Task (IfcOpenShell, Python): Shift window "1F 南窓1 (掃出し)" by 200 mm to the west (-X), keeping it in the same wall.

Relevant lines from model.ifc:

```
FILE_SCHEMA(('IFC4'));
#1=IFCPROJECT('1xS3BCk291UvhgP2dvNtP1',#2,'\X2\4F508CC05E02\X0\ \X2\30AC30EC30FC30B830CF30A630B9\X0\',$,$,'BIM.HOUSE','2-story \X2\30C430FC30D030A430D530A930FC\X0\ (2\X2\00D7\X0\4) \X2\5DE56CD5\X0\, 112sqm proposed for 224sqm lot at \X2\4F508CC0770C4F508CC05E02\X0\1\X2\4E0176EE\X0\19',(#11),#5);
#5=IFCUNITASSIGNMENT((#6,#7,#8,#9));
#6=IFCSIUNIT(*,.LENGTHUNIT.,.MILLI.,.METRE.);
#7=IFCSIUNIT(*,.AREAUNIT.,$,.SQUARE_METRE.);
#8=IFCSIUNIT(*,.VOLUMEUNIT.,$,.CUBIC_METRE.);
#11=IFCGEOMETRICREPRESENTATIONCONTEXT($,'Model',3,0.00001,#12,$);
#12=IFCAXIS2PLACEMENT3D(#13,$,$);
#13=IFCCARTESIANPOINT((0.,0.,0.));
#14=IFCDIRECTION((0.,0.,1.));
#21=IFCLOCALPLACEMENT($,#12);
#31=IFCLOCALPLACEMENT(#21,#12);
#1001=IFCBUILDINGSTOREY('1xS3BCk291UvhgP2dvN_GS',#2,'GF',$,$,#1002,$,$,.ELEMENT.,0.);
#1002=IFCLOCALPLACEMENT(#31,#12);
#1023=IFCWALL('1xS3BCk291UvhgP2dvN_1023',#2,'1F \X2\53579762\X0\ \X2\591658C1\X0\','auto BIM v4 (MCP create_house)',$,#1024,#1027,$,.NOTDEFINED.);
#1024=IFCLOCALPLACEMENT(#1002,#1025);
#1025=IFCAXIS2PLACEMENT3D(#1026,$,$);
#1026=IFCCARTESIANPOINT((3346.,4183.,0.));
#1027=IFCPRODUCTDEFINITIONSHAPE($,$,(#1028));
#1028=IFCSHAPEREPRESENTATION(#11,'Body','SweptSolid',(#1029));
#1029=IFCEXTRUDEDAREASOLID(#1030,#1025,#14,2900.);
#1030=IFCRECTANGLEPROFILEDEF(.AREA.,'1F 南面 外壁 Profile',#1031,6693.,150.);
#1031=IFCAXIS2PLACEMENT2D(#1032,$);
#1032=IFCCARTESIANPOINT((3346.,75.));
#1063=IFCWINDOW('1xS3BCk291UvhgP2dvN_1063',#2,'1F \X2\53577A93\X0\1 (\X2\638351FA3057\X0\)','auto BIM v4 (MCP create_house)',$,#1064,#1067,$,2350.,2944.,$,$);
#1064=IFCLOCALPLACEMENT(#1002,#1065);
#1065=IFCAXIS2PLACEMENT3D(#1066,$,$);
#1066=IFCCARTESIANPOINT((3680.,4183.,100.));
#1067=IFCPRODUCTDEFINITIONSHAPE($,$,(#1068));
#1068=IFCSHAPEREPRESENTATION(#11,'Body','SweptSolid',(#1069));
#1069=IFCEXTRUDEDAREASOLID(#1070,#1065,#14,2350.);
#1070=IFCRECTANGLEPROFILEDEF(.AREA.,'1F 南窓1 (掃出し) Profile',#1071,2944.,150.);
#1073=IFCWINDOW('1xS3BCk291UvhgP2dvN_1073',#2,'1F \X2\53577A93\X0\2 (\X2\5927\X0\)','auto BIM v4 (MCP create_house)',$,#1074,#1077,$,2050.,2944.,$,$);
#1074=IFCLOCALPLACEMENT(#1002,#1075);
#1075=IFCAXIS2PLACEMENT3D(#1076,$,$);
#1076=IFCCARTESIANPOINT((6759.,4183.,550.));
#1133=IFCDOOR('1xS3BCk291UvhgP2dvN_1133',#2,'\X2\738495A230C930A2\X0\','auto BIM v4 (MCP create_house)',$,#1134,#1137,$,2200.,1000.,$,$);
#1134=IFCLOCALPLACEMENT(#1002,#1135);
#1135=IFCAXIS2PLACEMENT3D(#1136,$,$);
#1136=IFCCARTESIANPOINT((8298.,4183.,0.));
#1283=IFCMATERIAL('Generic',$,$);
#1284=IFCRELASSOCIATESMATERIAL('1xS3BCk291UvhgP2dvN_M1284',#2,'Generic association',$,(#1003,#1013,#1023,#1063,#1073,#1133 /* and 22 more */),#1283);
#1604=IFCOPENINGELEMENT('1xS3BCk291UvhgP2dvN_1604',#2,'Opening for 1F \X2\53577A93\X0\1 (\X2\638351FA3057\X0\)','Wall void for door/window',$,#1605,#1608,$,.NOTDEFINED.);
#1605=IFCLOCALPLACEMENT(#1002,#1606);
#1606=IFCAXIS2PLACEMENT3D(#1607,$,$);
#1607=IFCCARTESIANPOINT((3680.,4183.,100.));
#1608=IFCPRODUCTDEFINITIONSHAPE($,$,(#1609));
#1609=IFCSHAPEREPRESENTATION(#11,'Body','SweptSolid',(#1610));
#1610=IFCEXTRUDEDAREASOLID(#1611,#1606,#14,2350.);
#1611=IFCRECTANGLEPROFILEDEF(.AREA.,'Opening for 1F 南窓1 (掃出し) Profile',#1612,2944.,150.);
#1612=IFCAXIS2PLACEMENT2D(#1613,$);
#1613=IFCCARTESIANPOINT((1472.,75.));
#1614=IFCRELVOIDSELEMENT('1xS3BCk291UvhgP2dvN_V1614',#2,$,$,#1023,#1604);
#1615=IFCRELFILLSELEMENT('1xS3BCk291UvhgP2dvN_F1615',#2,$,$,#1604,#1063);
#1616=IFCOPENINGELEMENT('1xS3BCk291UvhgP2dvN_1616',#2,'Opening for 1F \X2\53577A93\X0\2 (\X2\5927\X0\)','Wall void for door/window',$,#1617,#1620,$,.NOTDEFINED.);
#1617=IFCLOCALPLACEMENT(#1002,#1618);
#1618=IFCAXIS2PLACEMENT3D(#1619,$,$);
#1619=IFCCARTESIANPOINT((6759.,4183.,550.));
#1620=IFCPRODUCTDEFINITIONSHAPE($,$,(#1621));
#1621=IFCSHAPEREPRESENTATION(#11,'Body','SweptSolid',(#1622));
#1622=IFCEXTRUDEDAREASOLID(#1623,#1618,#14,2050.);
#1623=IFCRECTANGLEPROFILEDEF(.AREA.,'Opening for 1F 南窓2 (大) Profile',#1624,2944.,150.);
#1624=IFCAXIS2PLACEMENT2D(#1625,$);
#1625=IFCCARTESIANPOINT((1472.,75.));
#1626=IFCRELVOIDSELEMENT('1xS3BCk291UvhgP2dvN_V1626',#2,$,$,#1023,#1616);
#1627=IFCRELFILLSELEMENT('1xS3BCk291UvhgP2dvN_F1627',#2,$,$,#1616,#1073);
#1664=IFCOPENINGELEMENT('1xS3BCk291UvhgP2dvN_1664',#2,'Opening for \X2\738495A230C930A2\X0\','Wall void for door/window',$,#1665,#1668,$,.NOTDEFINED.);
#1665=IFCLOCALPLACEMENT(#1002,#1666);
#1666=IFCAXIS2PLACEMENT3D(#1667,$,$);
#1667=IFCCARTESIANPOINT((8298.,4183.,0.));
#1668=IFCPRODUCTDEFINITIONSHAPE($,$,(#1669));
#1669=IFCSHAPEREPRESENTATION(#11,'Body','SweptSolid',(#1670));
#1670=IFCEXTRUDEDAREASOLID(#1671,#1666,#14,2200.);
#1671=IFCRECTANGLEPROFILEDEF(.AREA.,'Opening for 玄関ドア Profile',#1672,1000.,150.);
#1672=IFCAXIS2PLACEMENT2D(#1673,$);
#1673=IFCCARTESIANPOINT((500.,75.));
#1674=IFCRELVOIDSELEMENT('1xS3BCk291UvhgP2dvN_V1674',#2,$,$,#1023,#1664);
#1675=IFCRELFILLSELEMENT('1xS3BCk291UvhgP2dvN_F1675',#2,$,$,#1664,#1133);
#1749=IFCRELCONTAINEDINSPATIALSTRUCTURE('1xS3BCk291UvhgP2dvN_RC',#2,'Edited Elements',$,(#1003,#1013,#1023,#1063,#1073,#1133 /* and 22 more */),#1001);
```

```python
import ifcopenshell
import ifcopenshell.api.geometry
import ifcopenshell.util.placement

model = ifcopenshell.open("model.ifc")

window = model.by_id(1063)
opening = window.FillsVoids[0].RelatingOpeningElement
wall = opening.VoidsElements[0].RelatingBuildingElement

wall_matrix = ifcopenshell.util.placement.get_local_placement(wall.ObjectPlacement)
shift = wall_matrix[:3, 0] * -200.0
before = ifcopenshell.util.placement.get_local_placement(window.ObjectPlacement)[:3, 3].copy()

# The window is not placed relative to its opening, so move both.
for product in (opening, window):
    matrix = ifcopenshell.util.placement.get_local_placement(product.ObjectPlacement)
    matrix[:3, 3] += shift
    ifcopenshell.api.geometry.edit_object_placement(model, product=product, matrix=matrix, is_si=False)

after = ifcopenshell.util.placement.get_local_placement(window.ObjectPlacement)[:3, 3]
print("window moved by", (after - before).round(3) + 0.0)

model.write("model_v2.ifc")
```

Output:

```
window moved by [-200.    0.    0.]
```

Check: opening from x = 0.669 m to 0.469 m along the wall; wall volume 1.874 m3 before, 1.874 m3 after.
